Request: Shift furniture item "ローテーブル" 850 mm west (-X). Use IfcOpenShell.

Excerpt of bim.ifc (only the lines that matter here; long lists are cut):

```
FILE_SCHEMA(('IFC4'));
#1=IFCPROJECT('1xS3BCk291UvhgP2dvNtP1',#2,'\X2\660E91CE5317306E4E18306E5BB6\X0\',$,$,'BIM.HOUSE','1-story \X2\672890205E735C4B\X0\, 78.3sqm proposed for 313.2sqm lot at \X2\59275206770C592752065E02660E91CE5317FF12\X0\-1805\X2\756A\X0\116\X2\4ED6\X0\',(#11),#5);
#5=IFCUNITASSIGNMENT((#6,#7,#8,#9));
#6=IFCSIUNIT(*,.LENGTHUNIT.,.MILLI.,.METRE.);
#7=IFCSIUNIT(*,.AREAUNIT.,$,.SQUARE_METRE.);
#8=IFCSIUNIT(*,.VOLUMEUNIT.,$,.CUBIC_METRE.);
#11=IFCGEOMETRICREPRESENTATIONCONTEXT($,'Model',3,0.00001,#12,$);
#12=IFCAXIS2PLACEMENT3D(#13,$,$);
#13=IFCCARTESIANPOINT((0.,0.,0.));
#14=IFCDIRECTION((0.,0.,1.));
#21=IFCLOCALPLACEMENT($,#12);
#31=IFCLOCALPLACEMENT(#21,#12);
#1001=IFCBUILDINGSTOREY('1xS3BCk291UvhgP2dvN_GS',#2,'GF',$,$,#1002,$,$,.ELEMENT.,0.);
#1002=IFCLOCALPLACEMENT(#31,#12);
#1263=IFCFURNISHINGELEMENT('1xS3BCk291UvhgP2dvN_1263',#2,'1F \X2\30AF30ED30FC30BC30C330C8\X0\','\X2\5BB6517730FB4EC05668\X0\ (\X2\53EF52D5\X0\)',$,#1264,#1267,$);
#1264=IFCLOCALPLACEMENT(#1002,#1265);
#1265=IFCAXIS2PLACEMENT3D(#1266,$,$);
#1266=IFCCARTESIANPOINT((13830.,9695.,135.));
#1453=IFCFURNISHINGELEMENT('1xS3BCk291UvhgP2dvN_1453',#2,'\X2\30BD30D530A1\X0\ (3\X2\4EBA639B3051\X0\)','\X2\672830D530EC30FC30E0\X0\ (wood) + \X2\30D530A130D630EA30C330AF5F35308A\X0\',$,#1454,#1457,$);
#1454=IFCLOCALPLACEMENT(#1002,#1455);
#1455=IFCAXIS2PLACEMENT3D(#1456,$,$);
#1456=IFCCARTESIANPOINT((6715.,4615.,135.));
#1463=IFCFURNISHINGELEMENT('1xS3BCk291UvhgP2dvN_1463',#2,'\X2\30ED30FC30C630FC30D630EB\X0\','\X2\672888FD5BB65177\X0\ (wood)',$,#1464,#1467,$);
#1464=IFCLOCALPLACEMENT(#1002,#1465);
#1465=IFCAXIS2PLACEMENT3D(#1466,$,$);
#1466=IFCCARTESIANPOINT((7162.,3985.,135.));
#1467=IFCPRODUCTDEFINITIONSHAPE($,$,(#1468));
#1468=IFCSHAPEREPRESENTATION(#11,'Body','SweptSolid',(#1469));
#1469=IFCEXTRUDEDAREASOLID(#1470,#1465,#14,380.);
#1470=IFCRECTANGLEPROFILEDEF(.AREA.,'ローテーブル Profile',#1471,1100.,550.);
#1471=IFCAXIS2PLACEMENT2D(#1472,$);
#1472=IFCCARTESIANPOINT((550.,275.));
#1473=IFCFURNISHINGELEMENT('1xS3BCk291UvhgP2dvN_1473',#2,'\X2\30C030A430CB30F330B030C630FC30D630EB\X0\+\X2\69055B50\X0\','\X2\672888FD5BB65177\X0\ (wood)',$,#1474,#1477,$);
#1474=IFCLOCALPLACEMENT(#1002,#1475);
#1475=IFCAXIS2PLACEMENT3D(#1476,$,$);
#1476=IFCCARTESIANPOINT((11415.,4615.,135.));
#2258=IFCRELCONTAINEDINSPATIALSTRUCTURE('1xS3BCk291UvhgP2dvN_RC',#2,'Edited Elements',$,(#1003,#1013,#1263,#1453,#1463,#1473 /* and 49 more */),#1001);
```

```python
import ifcopenshell
import ifcopenshell.api.geometry
import ifcopenshell.util.placement
import ifcopenshell.util.unit

model = ifcopenshell.open("bim.ifc")
unit_scale = ifcopenshell.util.unit.calculate_unit_scale(model)

item = model.by_guid("1xS3BCk291UvhgP2dvN_1463")
matrix = ifcopenshell.util.placement.get_local_placement(item.ObjectPlacement)
matrix[0, 3] -= 0.85 / unit_scale
ifcopenshell.api.geometry.edit_object_placement(model, product=item, matrix=matrix, is_si=False)

print(ifcopenshell.util.placement.get_local_placement(item.ObjectPlacement).round(3) + 0.0)

model.write("bim_rev.ifc")
```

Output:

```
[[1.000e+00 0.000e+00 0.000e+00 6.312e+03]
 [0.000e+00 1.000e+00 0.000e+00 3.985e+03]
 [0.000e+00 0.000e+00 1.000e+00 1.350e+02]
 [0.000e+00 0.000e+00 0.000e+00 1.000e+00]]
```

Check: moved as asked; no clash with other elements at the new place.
